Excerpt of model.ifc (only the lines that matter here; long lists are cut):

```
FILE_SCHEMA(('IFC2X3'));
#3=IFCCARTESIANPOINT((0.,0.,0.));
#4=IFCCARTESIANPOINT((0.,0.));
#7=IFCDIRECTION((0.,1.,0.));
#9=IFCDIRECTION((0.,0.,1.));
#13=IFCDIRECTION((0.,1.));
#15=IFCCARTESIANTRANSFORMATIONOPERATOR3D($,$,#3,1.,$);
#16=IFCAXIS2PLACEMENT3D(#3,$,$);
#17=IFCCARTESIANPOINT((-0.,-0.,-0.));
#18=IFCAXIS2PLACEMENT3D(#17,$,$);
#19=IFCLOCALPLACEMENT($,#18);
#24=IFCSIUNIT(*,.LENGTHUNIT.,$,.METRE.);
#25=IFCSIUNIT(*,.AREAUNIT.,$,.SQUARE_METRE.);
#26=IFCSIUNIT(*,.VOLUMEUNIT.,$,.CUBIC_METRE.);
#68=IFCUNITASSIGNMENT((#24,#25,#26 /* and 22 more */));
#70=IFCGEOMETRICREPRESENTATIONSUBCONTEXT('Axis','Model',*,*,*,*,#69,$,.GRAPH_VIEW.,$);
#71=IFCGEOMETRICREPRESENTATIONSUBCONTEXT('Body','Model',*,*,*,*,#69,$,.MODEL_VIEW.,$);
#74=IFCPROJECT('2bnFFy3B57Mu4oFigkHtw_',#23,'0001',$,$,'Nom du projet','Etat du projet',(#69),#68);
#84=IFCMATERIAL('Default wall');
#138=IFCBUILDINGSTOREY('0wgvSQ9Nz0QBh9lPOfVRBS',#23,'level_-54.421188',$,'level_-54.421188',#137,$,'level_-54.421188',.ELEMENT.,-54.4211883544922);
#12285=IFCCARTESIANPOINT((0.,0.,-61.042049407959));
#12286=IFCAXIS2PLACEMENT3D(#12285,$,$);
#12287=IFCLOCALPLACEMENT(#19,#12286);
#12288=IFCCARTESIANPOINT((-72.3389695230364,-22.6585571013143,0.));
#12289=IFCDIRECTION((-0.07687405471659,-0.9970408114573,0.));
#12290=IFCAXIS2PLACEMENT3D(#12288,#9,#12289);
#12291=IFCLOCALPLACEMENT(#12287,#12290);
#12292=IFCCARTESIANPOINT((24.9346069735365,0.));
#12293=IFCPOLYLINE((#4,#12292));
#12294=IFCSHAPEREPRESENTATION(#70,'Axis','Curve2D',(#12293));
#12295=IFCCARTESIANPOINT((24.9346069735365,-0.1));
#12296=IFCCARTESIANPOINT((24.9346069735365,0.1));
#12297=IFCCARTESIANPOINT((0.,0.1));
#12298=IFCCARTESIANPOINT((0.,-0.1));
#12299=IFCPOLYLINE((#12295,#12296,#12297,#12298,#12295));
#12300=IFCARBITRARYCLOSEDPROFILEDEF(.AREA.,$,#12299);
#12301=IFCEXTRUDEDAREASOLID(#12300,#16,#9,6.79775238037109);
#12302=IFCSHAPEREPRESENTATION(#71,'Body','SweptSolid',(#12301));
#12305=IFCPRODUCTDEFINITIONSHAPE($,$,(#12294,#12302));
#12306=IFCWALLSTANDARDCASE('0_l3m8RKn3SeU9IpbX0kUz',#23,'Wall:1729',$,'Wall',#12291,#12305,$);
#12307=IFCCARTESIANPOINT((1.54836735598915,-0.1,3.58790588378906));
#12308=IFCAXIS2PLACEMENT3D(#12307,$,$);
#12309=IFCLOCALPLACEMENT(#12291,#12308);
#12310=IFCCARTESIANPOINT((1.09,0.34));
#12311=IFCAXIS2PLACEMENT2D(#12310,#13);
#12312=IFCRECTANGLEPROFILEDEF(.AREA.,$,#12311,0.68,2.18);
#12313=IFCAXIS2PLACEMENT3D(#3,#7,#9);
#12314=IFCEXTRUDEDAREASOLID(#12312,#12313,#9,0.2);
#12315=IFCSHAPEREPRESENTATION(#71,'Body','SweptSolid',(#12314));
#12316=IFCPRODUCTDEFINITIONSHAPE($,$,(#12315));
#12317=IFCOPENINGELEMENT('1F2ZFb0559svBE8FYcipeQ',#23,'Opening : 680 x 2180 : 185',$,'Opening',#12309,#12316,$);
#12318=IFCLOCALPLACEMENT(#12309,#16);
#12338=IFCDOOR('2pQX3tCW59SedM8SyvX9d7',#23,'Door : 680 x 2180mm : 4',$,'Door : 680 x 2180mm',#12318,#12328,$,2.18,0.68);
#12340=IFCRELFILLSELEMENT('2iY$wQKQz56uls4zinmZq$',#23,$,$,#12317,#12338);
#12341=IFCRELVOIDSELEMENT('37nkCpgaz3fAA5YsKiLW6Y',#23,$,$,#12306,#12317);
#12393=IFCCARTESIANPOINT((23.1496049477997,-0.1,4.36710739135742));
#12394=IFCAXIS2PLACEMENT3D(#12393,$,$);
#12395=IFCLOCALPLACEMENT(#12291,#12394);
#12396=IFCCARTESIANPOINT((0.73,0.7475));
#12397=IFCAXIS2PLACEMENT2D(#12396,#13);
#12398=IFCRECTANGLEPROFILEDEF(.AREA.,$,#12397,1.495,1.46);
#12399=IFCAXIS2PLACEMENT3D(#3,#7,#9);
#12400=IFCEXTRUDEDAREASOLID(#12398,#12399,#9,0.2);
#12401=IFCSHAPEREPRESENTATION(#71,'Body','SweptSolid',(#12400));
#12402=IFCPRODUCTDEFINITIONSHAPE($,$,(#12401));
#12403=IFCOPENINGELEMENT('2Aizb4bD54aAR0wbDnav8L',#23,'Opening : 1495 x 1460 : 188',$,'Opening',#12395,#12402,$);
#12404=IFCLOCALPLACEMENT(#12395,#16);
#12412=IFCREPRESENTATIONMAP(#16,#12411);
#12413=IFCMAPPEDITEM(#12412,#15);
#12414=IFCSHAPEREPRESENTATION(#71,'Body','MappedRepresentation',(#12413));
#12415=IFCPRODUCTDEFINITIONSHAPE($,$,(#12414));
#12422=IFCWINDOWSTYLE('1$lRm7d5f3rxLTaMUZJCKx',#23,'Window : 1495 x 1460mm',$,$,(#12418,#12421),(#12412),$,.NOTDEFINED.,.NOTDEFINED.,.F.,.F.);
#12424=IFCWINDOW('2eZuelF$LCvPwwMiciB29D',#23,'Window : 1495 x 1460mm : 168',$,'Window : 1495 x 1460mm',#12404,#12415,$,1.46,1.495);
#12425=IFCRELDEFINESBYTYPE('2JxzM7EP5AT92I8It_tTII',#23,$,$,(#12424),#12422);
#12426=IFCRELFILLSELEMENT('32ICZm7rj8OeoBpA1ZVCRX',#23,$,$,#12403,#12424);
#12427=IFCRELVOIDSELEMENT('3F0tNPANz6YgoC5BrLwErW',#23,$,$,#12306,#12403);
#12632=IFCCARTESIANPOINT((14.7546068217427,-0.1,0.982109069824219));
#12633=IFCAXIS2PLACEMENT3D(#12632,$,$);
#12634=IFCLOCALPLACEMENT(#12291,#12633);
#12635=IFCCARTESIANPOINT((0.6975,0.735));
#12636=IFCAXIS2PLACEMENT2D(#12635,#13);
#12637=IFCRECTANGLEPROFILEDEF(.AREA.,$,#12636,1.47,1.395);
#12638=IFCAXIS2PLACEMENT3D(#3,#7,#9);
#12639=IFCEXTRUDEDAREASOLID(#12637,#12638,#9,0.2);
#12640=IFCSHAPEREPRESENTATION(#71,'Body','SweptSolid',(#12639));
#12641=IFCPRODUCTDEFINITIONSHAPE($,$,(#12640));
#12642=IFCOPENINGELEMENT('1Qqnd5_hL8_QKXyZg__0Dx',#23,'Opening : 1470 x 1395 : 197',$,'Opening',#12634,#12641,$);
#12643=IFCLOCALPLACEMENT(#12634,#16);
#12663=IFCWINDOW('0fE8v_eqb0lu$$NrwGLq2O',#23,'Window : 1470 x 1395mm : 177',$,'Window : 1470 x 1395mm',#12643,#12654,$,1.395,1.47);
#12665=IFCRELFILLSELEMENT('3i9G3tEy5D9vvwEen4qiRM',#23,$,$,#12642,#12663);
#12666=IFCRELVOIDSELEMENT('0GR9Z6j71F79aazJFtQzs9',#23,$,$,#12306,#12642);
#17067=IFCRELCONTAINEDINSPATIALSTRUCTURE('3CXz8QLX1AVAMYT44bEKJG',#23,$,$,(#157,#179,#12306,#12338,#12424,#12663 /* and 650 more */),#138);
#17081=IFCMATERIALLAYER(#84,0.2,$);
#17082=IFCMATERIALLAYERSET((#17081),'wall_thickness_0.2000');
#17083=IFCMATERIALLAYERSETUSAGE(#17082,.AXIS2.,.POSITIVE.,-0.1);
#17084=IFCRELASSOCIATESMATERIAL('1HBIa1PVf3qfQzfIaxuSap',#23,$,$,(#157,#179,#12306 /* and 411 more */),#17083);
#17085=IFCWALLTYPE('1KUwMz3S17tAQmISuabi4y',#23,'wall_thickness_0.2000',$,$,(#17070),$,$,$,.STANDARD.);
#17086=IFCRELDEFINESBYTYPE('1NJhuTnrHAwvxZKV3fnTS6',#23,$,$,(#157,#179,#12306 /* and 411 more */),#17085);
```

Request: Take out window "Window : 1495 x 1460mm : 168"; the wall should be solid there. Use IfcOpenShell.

```python
import ifcopenshell
import ifcopenshell.api.feature
import ifcopenshell.api.root
import ifcopenshell.geom
import ifcopenshell.util.shape

model = ifcopenshell.open("model.ifc")
settings = ifcopenshell.geom.settings()


def volume(element):
    """Net volume in cubic metres, openings subtracted."""
    shape = ifcopenshell.geom.create_shape(settings, element)
    return ifcopenshell.util.shape.get_volume(shape.geometry)


window = model.by_id(12424)
opening = window.FillsVoids[0].RelatingOpeningElement
wall = opening.VoidsElements[0].RelatingBuildingElement
before = volume(wall)

ifcopenshell.api.root.remove_product(model, product=window)
ifcopenshell.api.feature.remove_feature(model, feature=opening)

after = volume(wall)

print(f"wall volume {before:.3f} -> {after:.3f} m3")

model.write("model_rev.ifc")
```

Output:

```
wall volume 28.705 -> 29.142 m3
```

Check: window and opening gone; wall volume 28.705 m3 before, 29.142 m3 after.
